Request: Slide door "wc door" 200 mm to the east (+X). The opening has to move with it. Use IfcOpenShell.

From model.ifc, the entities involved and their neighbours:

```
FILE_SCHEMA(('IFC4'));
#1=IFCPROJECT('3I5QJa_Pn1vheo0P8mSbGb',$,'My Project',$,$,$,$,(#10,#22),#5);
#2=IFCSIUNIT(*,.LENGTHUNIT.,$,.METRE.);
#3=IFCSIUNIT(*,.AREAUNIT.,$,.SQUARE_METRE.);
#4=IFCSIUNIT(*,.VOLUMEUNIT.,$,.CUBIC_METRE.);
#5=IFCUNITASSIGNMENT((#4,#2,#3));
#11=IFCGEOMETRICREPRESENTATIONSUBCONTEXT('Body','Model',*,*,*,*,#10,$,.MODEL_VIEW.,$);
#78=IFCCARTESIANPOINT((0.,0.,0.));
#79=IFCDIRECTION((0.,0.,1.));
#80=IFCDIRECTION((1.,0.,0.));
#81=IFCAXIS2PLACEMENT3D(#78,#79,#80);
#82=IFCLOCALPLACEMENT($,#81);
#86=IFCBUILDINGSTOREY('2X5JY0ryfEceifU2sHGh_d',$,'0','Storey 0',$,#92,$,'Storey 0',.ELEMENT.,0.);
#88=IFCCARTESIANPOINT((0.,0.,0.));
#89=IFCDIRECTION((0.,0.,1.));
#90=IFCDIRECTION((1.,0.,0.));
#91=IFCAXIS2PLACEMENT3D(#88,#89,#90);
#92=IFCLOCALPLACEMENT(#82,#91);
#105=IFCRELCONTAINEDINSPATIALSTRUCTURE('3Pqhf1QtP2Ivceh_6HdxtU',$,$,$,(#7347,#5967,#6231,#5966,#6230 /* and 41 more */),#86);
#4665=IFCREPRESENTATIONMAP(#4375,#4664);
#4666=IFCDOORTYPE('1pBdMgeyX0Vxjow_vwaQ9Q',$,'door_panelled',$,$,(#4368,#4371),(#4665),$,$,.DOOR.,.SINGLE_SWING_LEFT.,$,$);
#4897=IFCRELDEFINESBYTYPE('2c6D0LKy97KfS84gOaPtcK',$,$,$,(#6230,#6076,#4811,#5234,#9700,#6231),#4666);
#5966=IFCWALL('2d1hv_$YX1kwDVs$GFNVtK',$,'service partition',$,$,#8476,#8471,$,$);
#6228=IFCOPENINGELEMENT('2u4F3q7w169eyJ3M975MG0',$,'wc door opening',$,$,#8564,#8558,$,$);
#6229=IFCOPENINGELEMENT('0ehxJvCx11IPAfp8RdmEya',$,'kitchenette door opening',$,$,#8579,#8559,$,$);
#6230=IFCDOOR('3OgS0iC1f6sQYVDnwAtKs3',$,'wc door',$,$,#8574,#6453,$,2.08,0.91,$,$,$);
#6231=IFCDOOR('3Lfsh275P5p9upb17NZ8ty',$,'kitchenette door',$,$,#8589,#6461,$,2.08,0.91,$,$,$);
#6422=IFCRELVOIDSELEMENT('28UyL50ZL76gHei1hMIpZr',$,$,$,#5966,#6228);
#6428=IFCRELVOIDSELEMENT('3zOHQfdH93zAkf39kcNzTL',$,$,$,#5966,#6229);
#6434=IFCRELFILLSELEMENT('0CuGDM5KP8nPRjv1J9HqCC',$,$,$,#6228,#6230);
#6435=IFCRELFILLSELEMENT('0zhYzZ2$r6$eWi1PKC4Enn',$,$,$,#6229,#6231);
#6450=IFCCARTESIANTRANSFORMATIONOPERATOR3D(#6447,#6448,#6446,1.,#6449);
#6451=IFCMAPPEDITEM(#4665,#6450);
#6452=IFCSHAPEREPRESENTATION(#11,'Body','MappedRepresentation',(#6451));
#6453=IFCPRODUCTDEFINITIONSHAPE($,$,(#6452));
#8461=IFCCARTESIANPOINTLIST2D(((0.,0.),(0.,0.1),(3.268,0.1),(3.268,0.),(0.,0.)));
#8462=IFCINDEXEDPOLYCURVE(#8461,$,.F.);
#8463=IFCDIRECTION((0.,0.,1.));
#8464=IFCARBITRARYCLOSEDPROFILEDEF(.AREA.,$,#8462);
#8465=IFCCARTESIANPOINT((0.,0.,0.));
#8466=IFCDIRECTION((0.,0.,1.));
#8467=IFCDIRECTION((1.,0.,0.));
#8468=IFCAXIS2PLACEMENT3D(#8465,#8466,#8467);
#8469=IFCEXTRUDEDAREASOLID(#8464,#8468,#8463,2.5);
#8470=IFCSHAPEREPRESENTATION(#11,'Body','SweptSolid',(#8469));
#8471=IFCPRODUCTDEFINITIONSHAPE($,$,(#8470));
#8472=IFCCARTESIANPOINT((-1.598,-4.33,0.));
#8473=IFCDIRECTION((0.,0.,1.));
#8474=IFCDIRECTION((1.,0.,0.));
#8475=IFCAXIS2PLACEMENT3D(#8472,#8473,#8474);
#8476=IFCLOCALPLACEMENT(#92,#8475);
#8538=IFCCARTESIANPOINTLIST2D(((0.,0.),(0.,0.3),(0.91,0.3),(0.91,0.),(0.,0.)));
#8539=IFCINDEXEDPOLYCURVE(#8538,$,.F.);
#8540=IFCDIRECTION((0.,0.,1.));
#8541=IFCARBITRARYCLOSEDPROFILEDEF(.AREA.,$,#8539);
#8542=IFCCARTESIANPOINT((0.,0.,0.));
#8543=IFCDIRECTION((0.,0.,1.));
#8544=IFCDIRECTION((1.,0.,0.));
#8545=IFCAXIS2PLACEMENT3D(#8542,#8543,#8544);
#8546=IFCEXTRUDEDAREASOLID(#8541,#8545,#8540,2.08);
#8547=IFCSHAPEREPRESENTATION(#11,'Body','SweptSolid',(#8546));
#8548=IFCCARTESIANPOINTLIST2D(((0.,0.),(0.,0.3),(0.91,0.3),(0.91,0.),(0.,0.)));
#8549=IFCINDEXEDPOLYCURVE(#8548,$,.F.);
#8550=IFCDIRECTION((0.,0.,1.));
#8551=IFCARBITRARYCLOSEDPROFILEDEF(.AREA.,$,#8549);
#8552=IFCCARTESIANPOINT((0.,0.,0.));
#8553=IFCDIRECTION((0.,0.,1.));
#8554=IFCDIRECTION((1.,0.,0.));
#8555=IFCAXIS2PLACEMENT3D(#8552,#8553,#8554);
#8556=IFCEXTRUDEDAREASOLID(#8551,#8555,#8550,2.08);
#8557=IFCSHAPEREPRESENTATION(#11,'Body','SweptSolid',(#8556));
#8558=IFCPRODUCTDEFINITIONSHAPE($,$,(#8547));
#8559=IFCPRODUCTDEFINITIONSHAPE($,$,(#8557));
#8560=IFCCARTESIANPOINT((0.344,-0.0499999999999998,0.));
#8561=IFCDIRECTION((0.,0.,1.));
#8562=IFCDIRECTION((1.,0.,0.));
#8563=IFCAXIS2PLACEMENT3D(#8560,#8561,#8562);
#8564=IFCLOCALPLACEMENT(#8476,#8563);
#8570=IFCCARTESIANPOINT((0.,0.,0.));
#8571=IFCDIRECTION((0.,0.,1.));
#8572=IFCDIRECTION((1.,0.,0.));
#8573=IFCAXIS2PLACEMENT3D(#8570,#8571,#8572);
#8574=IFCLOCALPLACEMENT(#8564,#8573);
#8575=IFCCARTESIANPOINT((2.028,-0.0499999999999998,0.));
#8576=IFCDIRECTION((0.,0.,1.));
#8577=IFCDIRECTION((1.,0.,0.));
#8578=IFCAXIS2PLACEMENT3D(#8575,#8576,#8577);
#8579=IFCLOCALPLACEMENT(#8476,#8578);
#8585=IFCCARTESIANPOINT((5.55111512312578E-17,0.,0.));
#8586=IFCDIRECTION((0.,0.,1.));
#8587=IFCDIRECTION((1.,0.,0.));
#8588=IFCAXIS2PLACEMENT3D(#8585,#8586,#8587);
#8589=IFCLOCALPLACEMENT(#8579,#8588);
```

```python
import ifcopenshell
import ifcopenshell.api.geometry
import ifcopenshell.util.placement

model = ifcopenshell.open("model.ifc")

door = model.by_id(6230)
opening = door.FillsVoids[0].RelatingOpeningElement
wall = opening.VoidsElements[0].RelatingBuildingElement

wall_matrix = ifcopenshell.util.placement.get_local_placement(wall.ObjectPlacement)
shift = wall_matrix[:3, 0] * 0.2
before = ifcopenshell.util.placement.get_local_placement(door.ObjectPlacement)[:3, 3].copy()

# The door is placed relative to its opening, so it follows when the opening moves.
matrix = ifcopenshell.util.placement.get_local_placement(opening.ObjectPlacement)
matrix[:3, 3] += shift
ifcopenshell.api.geometry.edit_object_placement(
    model, product=opening, matrix=matrix, is_si=False, should_transform_children=True
)

after = ifcopenshell.util.placement.get_local_placement(door.ObjectPlacement)[:3, 3]
print("door moved by", (after - before).round(3) + 0.0)

model.write("model-out.ifc")
```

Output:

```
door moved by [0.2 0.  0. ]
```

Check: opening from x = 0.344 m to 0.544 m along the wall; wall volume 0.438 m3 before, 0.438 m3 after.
